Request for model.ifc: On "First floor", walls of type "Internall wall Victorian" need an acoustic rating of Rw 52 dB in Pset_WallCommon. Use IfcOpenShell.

First a look at what the model holds.

```python
import ifcopenshell
import ifcopenshell.util.element

model = ifcopenshell.open("model.ifc")
print(model.schema)
storey = next(s for s in model.by_type("IfcBuildingStorey") if s.Name == "First floor")
walls = [e for e in ifcopenshell.util.element.get_decomposition(storey) if e.is_a("IfcWall")]
seen = {}
for e in walls:
    element_type = ifcopenshell.util.element.get_type(e)
    key = (element_type.Name if element_type != e and element_type else None, ifcopenshell.util.element.get_pset(e, "Pset_WallCommon", "AcousticRating"))
    seen[key] = seen.get(key, 0) + 1
for (name, value), count in sorted(seen.items(), key=str):
    print(count, "x", name, "|", value)
```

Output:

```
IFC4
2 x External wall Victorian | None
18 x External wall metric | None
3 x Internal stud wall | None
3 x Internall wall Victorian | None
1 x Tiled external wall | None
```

```python
import ifcopenshell
import ifcopenshell.api.pset
import ifcopenshell.util.element

model = ifcopenshell.open("model.ifc")

storey = next(s for s in model.by_type("IfcBuildingStorey") if s.Name == "First floor")
walls = [e for e in ifcopenshell.util.element.get_decomposition(storey) if e.is_a("IfcWall")]

count = 0
for e in walls:
    element_type = ifcopenshell.util.element.get_type(e)
    if element_type in (None, e) or element_type.Name != "Internall wall Victorian":
        continue
    # add_pset returns the element's existing set when there is one.
    pset = ifcopenshell.api.pset.add_pset(model, product=e, name="Pset_WallCommon")
    ifcopenshell.api.pset.edit_pset(model, pset=pset, properties={"AcousticRating": "Rw 52 dB"})
    count += 1

print(count, "walls updated")

model.write("model-out.ifc")
```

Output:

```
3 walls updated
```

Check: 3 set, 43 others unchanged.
